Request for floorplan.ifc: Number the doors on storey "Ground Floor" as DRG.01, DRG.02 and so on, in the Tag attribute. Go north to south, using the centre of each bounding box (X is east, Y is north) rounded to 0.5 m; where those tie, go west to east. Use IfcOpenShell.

First a look at what the model holds.

```python
import ifcopenshell
import ifcopenshell.util.element
import ifcopenshell.util.placement

model = ifcopenshell.open("floorplan.ifc")
print(model.schema)
storey = next(s for s in model.by_type("IfcBuildingStorey") if s.Name == "Ground Floor")
doors = [e for e in ifcopenshell.util.element.get_decomposition(storey) if e.is_a("IfcDoor")]
for e in sorted(doors, key=lambda e: e.id()):
    origin = ifcopenshell.util.placement.get_local_placement(e.ObjectPlacement)[:3, 3]
    print(e.id(), e.Tag, e.Name, origin.round(2) + 0.0, sep=" | ")
```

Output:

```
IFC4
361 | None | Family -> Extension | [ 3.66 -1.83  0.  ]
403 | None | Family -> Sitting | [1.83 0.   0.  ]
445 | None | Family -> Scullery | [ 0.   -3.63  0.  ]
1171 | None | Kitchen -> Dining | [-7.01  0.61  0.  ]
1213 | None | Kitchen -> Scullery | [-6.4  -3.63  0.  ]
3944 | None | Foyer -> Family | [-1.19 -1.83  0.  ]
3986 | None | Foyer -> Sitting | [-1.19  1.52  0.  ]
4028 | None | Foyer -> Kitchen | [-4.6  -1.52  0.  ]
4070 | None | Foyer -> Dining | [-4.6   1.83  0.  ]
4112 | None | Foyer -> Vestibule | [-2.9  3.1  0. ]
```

```python
import ifcopenshell
import ifcopenshell.geom
import ifcopenshell.util.element
import ifcopenshell.util.shape

model = ifcopenshell.open("floorplan.ifc")
settings = ifcopenshell.geom.settings()
settings.set("use-world-coords", True)


def centre(element):
    shape = ifcopenshell.geom.create_shape(settings, element)
    return ifcopenshell.util.shape.get_bbox_centroid(shape.geometry)


storey = next(s for s in model.by_type("IfcBuildingStorey") if s.Name == "Ground Floor")
doors = [e for e in ifcopenshell.util.element.get_decomposition(storey) if e.is_a("IfcDoor")]

# Insertion points can sit at a corner or the storey origin, so sort by the geometry (in metres).
centres = {e: centre(e) for e in doors}
doors.sort(key=lambda e: (-round(centres[e][1] / 0.5), centres[e][0]))

for i, e in enumerate(doors, start=1):
    number = f"DRG.{i:02d}"
    e.Tag = number
    print(e.id(), number)

model.write("floorplan_rev.ifc")
```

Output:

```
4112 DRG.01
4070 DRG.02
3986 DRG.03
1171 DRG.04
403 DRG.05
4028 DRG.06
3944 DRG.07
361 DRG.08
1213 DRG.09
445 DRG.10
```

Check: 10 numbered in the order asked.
